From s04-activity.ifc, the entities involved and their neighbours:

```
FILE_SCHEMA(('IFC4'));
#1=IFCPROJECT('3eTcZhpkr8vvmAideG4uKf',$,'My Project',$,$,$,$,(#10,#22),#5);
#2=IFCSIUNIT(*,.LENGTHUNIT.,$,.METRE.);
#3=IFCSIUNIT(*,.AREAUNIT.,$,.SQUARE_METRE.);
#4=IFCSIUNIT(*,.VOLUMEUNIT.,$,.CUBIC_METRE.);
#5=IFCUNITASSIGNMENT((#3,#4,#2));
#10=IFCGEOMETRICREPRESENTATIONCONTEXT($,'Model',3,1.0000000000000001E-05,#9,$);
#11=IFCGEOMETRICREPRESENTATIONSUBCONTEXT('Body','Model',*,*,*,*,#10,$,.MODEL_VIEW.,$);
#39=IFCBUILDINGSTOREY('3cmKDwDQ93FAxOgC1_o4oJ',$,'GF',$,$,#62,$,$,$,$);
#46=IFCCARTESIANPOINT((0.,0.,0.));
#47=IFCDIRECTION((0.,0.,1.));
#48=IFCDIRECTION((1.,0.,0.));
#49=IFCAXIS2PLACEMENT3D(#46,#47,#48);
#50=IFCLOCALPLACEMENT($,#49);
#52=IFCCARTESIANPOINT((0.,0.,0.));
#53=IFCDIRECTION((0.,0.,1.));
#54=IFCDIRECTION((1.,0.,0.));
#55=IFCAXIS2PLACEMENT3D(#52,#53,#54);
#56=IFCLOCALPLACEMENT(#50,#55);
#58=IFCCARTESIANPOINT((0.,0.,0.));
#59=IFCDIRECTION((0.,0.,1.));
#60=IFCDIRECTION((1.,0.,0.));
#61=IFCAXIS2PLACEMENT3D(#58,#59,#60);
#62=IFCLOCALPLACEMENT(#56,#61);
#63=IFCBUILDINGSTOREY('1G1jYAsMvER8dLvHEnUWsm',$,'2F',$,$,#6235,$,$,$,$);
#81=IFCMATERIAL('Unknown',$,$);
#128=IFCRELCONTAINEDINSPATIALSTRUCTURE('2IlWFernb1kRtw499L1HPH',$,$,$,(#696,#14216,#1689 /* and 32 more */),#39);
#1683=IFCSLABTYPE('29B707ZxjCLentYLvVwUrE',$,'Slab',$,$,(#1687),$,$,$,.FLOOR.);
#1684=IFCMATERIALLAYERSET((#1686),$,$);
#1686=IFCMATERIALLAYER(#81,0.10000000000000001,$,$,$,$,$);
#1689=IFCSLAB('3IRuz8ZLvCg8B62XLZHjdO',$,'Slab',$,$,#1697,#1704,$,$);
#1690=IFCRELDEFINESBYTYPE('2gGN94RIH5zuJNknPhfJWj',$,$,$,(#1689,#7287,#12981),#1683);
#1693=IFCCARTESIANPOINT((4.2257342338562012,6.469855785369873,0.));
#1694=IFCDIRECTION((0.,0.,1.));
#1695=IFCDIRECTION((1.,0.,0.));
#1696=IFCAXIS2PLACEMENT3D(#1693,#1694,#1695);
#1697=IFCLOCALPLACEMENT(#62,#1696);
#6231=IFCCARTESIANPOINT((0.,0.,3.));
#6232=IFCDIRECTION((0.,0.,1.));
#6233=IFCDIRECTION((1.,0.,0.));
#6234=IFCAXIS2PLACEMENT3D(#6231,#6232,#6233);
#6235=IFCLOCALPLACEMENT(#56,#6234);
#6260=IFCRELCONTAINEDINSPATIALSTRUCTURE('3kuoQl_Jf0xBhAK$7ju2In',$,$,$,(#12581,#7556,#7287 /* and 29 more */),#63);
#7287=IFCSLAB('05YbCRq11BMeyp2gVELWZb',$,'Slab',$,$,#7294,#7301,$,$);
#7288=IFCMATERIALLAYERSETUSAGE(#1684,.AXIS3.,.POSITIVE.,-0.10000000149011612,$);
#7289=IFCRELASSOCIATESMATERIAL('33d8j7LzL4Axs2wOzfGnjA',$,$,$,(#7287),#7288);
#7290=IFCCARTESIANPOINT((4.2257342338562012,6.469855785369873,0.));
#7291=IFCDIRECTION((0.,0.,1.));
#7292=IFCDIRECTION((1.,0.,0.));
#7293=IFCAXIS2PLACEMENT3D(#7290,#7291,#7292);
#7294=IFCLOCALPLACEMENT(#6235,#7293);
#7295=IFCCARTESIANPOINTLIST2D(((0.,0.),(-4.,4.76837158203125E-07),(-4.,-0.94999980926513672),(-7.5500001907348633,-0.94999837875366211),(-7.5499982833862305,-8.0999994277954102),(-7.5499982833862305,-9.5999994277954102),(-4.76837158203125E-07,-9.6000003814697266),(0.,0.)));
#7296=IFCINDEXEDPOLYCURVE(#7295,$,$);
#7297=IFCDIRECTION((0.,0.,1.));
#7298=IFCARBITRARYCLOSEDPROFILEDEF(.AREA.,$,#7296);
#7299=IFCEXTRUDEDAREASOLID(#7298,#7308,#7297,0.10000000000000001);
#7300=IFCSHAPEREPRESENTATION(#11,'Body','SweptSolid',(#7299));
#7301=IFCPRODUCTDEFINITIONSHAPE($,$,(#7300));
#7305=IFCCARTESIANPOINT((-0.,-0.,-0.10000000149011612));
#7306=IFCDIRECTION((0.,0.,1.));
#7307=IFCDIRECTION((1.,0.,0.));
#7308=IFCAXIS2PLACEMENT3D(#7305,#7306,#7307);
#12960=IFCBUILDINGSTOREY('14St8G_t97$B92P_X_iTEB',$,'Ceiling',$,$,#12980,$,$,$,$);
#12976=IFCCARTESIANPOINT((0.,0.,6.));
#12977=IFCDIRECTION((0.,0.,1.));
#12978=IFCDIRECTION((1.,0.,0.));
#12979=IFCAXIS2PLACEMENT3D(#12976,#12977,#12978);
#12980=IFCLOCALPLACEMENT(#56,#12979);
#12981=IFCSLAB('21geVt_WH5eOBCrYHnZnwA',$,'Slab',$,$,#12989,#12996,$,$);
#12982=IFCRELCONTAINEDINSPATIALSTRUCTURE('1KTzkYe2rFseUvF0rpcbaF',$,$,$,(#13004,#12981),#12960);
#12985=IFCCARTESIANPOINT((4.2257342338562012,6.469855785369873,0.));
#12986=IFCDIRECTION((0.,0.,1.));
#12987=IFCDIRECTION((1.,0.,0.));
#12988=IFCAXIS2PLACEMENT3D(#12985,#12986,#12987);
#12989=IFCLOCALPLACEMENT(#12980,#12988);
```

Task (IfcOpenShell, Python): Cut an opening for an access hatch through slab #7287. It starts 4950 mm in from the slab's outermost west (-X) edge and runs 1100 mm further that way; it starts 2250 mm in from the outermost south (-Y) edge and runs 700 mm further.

```python
import numpy as np
import ifcopenshell
import ifcopenshell.api.feature
import ifcopenshell.api.geometry
import ifcopenshell.api.root
import ifcopenshell.geom
import ifcopenshell.util.placement
import ifcopenshell.util.representation
import ifcopenshell.util.shape
import ifcopenshell.util.unit

model = ifcopenshell.open("s04-activity.ifc")
unit_scale = ifcopenshell.util.unit.calculate_unit_scale(model)
settings = ifcopenshell.geom.settings()


def volume(element):
    """Net volume in cubic metres, openings subtracted."""
    shape = ifcopenshell.geom.create_shape(settings, element)
    return ifcopenshell.util.shape.get_volume(shape.geometry)


slab = model.by_id(7287)
before = volume(slab)

# Extent in the slab's own axes, in metres. The edges named are its -X and -Y sides.
slab_shape = ifcopenshell.geom.create_shape(settings, slab)
vertices = ifcopenshell.util.shape.get_vertices(slab_shape.geometry)
x_min, y_min, bottom = vertices.min(axis=0)
top = vertices[:, 2].max()

opening = ifcopenshell.api.root.create_entity(model, ifc_class="IfcOpeningElement", name="Access hatch opening", predefined_type="OPENING")
context = ifcopenshell.util.representation.get_context(model, "Model", "Body", "MODEL_VIEW")
width, depth = 1.1, 0.7
outline = [(0.0, 0.0), (width, 0.0), (width, depth), (0.0, depth), (0.0, 0.0)]
# Overshoot both faces by 50 mm so the cut is clean.
shape = ifcopenshell.api.geometry.add_slab_representation(
    model, context=context, depth=top - bottom + 0.1, polyline=outline
)
ifcopenshell.api.geometry.assign_representation(model, product=opening, representation=shape)

matrix = ifcopenshell.util.placement.get_local_placement(slab.ObjectPlacement)
matrix[:, 3] = matrix @ np.append(np.array([x_min + 4.95, y_min + 2.25, bottom - 0.05]) / unit_scale, 1.0)
ifcopenshell.api.geometry.edit_object_placement(model, product=opening, matrix=matrix, is_si=False)
ifcopenshell.api.feature.add_feature(model, feature=opening, element=slab)

after = volume(slab)

print(f"slab volume {before:.3f} -> {after:.3f} m3")

model.write("s04-activity_updated.ifc")
```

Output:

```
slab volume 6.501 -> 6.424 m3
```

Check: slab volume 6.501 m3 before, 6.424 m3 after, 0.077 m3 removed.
